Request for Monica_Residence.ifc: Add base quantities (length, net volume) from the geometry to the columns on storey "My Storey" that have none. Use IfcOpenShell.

First a look at what the model holds.

```python
import ifcopenshell
import ifcopenshell.util.element
import ifcopenshell.util.unit

model = ifcopenshell.open("Monica_Residence.ifc")
print(model.schema)
for unit_type in ("LENGTHUNIT", "AREAUNIT", "VOLUMEUNIT"):
    print(unit_type, ifcopenshell.util.unit.calculate_unit_scale(model, unit_type))
storey = next(s for s in model.by_type("IfcBuildingStorey") if s.Name == "My Storey")
columns = [e for e in ifcopenshell.util.element.get_decomposition(storey) if e.is_a("IfcColumn")]
for e in sorted(columns, key=lambda e: e.id()):
    print(e.id(), e.is_a(), e.Name, list(ifcopenshell.util.element.get_psets(e, qtos_only=True)), sep=" | ")
```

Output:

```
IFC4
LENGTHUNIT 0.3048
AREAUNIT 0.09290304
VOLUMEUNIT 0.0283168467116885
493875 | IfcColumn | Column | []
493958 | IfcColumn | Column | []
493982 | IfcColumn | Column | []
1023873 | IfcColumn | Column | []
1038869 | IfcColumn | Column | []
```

```python
import ifcopenshell
import ifcopenshell.api.pset
import ifcopenshell.geom
import ifcopenshell.util.element
import ifcopenshell.util.shape
import ifcopenshell.util.unit

model = ifcopenshell.open("Monica_Residence.ifc")
unit_scale = ifcopenshell.util.unit.calculate_unit_scale(model)
volume_scale = ifcopenshell.util.unit.calculate_unit_scale(model, "VOLUMEUNIT")
settings = ifcopenshell.geom.settings()

storey = next(s for s in model.by_type("IfcBuildingStorey") if s.Name == "My Storey")
columns = [e for e in ifcopenshell.util.element.get_decomposition(storey) if e.is_a("IfcColumn")]

for e in sorted(columns, key=lambda e: e.id()):
    if ifcopenshell.util.element.get_psets(e, qtos_only=True, should_inherit=False):
        continue
    # Geometry comes back in metres, in the element's own axes.
    shape = ifcopenshell.geom.create_shape(settings, e)
    values = {
        "Length": ifcopenshell.util.shape.get_z(shape.geometry) / unit_scale,
        "NetVolume": ifcopenshell.util.shape.get_volume(shape.geometry) / volume_scale,
    }
    qto = ifcopenshell.api.pset.add_qto(model, product=e, name="Qto_ColumnBaseQuantities")
    ifcopenshell.api.pset.edit_qto(model, qto=qto, properties=values)
    print(e.id(), {k: round(v, 3) for k, v in values.items()})

model.write("Monica_Residence_edited.ifc")
```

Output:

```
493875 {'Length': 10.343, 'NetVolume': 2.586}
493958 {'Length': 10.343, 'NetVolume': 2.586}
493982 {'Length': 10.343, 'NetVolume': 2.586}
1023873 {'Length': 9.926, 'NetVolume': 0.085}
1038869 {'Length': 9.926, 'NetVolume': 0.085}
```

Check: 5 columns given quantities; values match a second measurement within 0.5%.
